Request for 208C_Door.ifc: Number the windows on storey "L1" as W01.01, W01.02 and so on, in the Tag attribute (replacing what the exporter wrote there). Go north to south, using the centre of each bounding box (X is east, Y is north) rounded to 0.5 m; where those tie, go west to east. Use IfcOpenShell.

First a look at what the model holds.

```python
import ifcopenshell
import ifcopenshell.util.element
import ifcopenshell.util.placement

model = ifcopenshell.open("208C_Door.ifc")
print(model.schema)
storey = next(s for s in model.by_type("IfcBuildingStorey") if s.Name == "L1")
windows = [e for e in ifcopenshell.util.element.get_decomposition(storey) if e.is_a("IfcWindow")]
for e in sorted(windows, key=lambda e: e.id()):
    origin = ifcopenshell.util.placement.get_local_placement(e.ObjectPlacement)[:3, 3]
    print(e.id(), e.Tag, e.Name, origin.round(2) + 0.0, sep=" | ")
```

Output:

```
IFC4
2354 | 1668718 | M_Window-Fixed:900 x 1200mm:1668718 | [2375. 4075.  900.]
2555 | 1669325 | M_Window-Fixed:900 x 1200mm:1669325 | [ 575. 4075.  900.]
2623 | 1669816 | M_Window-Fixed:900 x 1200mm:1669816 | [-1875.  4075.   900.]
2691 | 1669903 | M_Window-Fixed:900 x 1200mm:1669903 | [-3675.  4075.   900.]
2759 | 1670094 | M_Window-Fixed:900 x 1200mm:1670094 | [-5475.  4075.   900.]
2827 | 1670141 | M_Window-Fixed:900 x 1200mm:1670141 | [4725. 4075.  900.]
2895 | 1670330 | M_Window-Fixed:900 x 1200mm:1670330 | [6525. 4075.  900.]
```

```python
import ifcopenshell
import ifcopenshell.geom
import ifcopenshell.util.element
import ifcopenshell.util.shape

model = ifcopenshell.open("208C_Door.ifc")
settings = ifcopenshell.geom.settings()
settings.set("use-world-coords", True)


def centre(element):
    shape = ifcopenshell.geom.create_shape(settings, element)
    return ifcopenshell.util.shape.get_bbox_centroid(shape.geometry)


storey = next(s for s in model.by_type("IfcBuildingStorey") if s.Name == "L1")
windows = [e for e in ifcopenshell.util.element.get_decomposition(storey) if e.is_a("IfcWindow")]

# Insertion points can sit at a corner or the storey origin, so sort by the geometry (in metres).
centres = {e: centre(e) for e in windows}
windows.sort(key=lambda e: (-round(centres[e][1] / 0.5), centres[e][0]))

for i, e in enumerate(windows, start=1):
    number = f"W01.{i:02d}"
    e.Tag = number
    print(e.id(), number)

model.write("208C_Door_v2.ifc")
```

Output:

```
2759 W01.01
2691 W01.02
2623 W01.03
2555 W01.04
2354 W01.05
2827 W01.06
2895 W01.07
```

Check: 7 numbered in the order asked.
